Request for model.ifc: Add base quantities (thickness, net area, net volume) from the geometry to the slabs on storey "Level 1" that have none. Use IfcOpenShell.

First a look at what the model holds.

```python
import ifcopenshell
import ifcopenshell.util.element
import ifcopenshell.util.unit

model = ifcopenshell.open("model.ifc")
print(model.schema)
for unit_type in ("LENGTHUNIT", "AREAUNIT", "VOLUMEUNIT"):
    print(unit_type, ifcopenshell.util.unit.calculate_unit_scale(model, unit_type))
storey = next(s for s in model.by_type("IfcBuildingStorey") if s.Name == "Level 1")
slabs = [e for e in ifcopenshell.util.element.get_decomposition(storey) if e.is_a("IfcSlab")]
for e in sorted(slabs, key=lambda e: e.id()):
    print(e.id(), e.is_a(), e.Name, list(ifcopenshell.util.element.get_psets(e, qtos_only=True)), sep=" | ")
```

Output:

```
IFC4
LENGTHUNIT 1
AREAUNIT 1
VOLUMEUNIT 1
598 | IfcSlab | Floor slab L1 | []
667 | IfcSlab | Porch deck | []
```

```python
import ifcopenshell
import ifcopenshell.api.pset
import ifcopenshell.geom
import ifcopenshell.util.element
import ifcopenshell.util.shape
import ifcopenshell.util.unit

model = ifcopenshell.open("model.ifc")
unit_scale = ifcopenshell.util.unit.calculate_unit_scale(model)
area_scale = ifcopenshell.util.unit.calculate_unit_scale(model, "AREAUNIT")
volume_scale = ifcopenshell.util.unit.calculate_unit_scale(model, "VOLUMEUNIT")
settings = ifcopenshell.geom.settings()

storey = next(s for s in model.by_type("IfcBuildingStorey") if s.Name == "Level 1")
slabs = [e for e in ifcopenshell.util.element.get_decomposition(storey) if e.is_a("IfcSlab")]

for e in sorted(slabs, key=lambda e: e.id()):
    if ifcopenshell.util.element.get_psets(e, qtos_only=True, should_inherit=False):
        continue
    # Geometry comes back in metres, in the element's own axes.
    shape = ifcopenshell.geom.create_shape(settings, e)
    values = {
        "Width": ifcopenshell.util.shape.get_z(shape.geometry) / unit_scale,
        "NetArea": ifcopenshell.util.shape.get_footprint_area(shape.geometry) / area_scale,
        "NetVolume": ifcopenshell.util.shape.get_volume(shape.geometry) / volume_scale,
    }
    qto = ifcopenshell.api.pset.add_qto(model, product=e, name="Qto_SlabBaseQuantities")
    ifcopenshell.api.pset.edit_qto(model, qto=qto, properties=values)
    print(e.id(), {k: round(v, 3) for k, v in values.items()})

model.write("model_v2.ifc")
```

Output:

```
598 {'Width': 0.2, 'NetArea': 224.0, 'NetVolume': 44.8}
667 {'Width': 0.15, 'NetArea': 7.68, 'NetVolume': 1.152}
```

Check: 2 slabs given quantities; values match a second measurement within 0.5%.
